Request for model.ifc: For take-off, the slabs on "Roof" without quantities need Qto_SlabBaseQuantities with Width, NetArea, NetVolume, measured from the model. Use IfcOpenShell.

First a look at what the model holds.

```python
import ifcopenshell
import ifcopenshell.util.element
import ifcopenshell.util.unit

model = ifcopenshell.open("model.ifc")
print(model.schema)
for unit_type in ("LENGTHUNIT", "AREAUNIT", "VOLUMEUNIT"):
    print(unit_type, ifcopenshell.util.unit.calculate_unit_scale(model, unit_type))
storey = next(s for s in model.by_type("IfcBuildingStorey") if s.Name == "Roof")
slabs = [e for e in ifcopenshell.util.element.get_decomposition(storey) if e.is_a("IfcSlab")]
for e in sorted(slabs, key=lambda e: e.id()):
    print(e.id(), e.is_a(), e.Name, list(ifcopenshell.util.element.get_psets(e, qtos_only=True)), sep=" | ")
```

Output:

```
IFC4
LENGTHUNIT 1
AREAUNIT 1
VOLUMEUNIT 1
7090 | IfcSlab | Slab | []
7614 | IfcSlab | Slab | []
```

```python
import ifcopenshell
import ifcopenshell.api.pset
import ifcopenshell.geom
import ifcopenshell.util.element
import ifcopenshell.util.shape
import ifcopenshell.util.unit

model = ifcopenshell.open("model.ifc")
unit_scale = ifcopenshell.util.unit.calculate_unit_scale(model)
area_scale = ifcopenshell.util.unit.calculate_unit_scale(model, "AREAUNIT")
volume_scale = ifcopenshell.util.unit.calculate_unit_scale(model, "VOLUMEUNIT")
settings = ifcopenshell.geom.settings()

storey = next(s for s in model.by_type("IfcBuildingStorey") if s.Name == "Roof")
slabs = [e for e in ifcopenshell.util.element.get_decomposition(storey) if e.is_a("IfcSlab")]

for e in sorted(slabs, key=lambda e: e.id()):
    if ifcopenshell.util.element.get_psets(e, qtos_only=True, should_inherit=False):
        continue
    # Geometry comes back in metres, in the element's own axes.
    shape = ifcopenshell.geom.create_shape(settings, e)
    values = {
        "Width": ifcopenshell.util.shape.get_z(shape.geometry) / unit_scale,
        "NetArea": ifcopenshell.util.shape.get_footprint_area(shape.geometry) / area_scale,
        "NetVolume": ifcopenshell.util.shape.get_volume(shape.geometry) / volume_scale,
    }
    qto = ifcopenshell.api.pset.add_qto(model, product=e, name="Qto_SlabBaseQuantities")
    ifcopenshell.api.pset.edit_qto(model, qto=qto, properties=values)
    print(e.id(), {k: round(v, 3) for k, v in values.items()})

model.write("model_v2.ifc")
```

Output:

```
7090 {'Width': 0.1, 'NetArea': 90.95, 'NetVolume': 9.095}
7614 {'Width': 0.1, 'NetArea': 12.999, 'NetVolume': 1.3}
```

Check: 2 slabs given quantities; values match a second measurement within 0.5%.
